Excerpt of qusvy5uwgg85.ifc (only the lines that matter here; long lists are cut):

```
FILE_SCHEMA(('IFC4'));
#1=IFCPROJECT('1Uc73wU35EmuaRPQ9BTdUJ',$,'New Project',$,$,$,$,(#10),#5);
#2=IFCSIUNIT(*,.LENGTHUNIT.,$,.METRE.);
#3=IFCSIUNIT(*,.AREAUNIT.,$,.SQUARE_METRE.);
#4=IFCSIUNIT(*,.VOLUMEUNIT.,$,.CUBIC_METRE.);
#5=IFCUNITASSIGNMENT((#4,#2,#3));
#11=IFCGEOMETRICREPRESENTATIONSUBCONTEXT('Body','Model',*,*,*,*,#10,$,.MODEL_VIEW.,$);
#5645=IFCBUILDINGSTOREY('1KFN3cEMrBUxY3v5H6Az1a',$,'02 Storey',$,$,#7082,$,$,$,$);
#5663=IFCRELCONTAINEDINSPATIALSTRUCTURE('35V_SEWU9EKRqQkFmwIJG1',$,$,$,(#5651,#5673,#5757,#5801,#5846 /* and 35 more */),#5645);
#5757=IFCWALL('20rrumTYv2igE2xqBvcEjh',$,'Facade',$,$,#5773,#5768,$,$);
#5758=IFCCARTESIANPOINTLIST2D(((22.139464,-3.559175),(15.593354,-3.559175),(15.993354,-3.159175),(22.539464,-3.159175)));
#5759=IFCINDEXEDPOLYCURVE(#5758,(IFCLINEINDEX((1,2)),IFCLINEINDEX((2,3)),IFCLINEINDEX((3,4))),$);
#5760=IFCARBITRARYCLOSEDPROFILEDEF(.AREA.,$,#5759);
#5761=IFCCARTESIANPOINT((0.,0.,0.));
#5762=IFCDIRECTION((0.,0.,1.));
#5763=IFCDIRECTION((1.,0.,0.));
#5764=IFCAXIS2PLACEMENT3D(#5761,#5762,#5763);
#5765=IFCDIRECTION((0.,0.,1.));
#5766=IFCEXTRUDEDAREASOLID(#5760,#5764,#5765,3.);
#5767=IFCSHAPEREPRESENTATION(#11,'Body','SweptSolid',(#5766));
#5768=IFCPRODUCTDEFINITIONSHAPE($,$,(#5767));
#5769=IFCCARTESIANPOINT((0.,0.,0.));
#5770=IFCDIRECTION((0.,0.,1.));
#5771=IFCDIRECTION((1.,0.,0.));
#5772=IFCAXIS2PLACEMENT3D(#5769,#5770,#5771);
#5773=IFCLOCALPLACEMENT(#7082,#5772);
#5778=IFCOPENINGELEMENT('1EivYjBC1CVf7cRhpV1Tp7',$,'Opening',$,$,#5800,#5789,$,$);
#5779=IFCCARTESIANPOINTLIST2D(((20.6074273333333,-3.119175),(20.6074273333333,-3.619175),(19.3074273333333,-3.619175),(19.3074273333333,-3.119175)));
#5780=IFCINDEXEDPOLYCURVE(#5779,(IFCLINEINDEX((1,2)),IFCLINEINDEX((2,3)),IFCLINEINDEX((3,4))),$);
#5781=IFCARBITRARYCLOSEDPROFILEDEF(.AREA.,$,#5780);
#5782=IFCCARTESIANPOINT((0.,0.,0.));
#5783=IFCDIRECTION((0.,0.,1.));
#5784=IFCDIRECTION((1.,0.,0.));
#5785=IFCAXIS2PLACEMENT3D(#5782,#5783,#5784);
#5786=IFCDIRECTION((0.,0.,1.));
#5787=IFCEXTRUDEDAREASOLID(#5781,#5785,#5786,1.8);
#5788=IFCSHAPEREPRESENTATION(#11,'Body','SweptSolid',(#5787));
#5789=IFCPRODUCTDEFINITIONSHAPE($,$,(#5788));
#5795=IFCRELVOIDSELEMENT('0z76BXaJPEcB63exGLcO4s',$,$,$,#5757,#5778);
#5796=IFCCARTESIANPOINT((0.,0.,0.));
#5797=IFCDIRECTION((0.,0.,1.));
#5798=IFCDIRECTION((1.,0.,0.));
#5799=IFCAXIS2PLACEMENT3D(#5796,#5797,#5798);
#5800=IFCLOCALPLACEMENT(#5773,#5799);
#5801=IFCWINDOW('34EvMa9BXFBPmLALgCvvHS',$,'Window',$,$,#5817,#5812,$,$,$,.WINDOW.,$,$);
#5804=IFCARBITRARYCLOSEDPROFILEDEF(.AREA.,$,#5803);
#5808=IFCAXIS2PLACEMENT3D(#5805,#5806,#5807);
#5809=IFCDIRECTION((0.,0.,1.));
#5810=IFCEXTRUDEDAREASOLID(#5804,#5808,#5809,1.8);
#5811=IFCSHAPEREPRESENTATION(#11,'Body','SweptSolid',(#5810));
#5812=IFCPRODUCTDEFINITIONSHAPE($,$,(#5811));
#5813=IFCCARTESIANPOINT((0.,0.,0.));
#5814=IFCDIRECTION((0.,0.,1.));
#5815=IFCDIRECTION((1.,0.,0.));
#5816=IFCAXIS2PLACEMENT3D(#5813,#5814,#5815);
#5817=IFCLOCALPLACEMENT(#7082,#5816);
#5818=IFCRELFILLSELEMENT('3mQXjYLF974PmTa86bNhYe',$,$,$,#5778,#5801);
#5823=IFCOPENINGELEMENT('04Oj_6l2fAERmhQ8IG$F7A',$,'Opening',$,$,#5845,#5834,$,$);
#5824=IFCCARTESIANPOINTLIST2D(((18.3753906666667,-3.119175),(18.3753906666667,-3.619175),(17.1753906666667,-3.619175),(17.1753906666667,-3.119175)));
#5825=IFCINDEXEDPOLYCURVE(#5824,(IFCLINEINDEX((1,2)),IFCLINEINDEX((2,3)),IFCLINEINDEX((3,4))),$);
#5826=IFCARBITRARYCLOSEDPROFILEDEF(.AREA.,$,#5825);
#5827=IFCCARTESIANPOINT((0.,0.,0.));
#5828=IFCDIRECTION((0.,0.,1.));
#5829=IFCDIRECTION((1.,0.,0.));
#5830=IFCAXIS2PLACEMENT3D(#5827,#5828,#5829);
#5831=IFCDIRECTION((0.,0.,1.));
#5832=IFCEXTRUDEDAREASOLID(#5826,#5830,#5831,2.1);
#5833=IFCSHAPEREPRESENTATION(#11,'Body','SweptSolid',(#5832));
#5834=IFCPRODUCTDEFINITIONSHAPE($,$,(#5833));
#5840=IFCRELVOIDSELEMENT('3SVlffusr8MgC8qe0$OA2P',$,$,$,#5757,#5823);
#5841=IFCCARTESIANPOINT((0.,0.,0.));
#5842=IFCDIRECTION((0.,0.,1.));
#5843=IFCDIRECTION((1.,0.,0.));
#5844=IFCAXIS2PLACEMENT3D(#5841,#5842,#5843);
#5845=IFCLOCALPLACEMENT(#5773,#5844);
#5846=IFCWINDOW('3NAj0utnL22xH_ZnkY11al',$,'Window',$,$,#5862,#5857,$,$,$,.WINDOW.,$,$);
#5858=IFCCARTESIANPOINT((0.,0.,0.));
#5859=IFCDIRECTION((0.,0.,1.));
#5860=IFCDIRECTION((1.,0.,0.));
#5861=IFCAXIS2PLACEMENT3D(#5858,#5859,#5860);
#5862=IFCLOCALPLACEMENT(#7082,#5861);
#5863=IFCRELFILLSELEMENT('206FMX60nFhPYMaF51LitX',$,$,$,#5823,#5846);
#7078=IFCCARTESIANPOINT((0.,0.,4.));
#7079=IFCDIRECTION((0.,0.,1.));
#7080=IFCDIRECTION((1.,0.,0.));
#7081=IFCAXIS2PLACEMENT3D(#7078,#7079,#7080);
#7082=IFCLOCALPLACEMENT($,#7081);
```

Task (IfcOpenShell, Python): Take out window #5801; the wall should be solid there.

```python
import ifcopenshell
import ifcopenshell.api.feature
import ifcopenshell.api.root
import ifcopenshell.geom
import ifcopenshell.util.shape

model = ifcopenshell.open("qusvy5uwgg85.ifc")
settings = ifcopenshell.geom.settings()


def volume(element):
    """Net volume in cubic metres, openings subtracted."""
    shape = ifcopenshell.geom.create_shape(settings, element)
    return ifcopenshell.util.shape.get_volume(shape.geometry)


window = model.by_id(5801)
opening = window.FillsVoids[0].RelatingOpeningElement
wall = opening.VoidsElements[0].RelatingBuildingElement
before = volume(wall)

ifcopenshell.api.root.remove_product(model, product=window)
ifcopenshell.api.feature.remove_feature(model, feature=opening)

after = volume(wall)

print(f"wall volume {before:.3f} -> {after:.3f} m3")

model.write("qusvy5uwgg85-out.ifc")
```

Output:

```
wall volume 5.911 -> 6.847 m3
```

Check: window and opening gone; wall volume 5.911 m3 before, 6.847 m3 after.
